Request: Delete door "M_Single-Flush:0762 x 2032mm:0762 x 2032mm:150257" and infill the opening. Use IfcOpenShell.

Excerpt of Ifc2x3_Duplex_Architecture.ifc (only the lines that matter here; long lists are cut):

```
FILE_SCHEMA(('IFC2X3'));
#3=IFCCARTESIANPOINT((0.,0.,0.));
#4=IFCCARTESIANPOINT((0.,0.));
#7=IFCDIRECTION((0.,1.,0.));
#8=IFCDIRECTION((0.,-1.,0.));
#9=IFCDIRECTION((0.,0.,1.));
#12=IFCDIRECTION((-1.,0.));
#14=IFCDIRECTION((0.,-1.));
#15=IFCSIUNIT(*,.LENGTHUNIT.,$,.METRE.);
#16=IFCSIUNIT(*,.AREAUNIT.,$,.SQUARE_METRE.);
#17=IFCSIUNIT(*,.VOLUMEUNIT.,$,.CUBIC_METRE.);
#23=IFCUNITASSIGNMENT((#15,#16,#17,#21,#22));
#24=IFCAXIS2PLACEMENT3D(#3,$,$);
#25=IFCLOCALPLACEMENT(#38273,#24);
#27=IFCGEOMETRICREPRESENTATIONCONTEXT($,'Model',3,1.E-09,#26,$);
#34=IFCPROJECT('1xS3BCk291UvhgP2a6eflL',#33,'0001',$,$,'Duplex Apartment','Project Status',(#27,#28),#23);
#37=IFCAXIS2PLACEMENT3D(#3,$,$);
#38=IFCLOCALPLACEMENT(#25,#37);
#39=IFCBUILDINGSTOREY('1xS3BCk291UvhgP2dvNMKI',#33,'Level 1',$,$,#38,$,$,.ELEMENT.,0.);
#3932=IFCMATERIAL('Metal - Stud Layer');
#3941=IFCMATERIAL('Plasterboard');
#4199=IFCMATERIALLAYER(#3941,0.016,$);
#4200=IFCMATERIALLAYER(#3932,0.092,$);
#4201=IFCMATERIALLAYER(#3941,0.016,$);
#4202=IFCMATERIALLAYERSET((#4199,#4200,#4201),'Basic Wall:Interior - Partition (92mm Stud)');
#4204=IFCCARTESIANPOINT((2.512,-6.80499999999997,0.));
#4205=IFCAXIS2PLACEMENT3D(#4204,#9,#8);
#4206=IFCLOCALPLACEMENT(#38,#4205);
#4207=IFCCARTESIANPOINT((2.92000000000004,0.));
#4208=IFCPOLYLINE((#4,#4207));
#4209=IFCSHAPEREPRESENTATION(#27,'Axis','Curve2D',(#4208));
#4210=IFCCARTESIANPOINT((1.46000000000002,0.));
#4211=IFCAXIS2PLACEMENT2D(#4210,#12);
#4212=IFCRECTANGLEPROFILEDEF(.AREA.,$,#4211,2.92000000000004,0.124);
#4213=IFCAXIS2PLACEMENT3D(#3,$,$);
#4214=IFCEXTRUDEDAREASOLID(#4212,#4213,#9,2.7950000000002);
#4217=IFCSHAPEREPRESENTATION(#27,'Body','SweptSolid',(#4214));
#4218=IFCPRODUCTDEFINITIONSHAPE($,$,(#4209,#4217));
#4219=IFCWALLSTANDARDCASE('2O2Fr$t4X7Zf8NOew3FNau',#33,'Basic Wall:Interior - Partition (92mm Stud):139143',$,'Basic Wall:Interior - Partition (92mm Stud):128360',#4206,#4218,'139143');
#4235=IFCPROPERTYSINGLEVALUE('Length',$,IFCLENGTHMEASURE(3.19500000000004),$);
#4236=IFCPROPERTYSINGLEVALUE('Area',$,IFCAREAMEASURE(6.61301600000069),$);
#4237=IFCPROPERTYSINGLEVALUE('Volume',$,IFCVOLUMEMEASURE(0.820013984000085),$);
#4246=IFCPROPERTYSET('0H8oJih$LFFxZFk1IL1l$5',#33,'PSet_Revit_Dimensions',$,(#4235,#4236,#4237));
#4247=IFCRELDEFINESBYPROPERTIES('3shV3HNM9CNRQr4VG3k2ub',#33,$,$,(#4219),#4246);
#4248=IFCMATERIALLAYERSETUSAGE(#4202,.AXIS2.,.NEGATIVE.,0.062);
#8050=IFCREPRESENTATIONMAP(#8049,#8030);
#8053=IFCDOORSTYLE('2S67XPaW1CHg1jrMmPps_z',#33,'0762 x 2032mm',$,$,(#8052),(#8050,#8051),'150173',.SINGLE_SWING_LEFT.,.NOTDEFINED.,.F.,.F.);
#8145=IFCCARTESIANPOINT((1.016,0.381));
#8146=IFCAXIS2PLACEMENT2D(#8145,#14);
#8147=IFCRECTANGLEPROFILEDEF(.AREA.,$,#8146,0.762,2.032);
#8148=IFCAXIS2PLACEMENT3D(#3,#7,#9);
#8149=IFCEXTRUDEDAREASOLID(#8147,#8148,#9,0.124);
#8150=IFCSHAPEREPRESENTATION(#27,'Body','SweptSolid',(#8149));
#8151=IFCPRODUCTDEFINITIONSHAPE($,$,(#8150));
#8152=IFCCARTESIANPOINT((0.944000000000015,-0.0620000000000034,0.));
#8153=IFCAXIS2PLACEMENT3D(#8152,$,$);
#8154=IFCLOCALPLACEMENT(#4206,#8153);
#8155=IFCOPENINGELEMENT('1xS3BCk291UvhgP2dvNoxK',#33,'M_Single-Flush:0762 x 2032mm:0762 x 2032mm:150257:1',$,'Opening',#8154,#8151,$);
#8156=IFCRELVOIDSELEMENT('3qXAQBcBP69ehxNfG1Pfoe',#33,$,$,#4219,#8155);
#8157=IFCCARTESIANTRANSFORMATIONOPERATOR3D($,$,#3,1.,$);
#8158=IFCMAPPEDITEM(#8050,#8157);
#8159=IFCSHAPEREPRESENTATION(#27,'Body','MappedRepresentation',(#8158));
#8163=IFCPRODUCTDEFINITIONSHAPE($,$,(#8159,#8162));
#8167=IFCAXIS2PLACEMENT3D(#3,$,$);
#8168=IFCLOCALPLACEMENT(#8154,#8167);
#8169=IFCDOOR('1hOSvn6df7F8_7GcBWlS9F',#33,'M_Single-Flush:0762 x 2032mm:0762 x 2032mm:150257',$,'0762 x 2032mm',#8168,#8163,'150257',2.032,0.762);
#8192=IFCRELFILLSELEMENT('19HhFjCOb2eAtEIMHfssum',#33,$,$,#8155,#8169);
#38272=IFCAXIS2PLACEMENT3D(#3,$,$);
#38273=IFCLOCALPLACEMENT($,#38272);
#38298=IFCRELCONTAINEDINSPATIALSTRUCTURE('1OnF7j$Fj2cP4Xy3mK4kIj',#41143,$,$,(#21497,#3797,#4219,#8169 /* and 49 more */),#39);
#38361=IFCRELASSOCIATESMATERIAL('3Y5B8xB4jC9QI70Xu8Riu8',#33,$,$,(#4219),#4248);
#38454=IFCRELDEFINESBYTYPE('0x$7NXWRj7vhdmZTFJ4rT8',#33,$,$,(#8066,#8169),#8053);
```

```python
import ifcopenshell
import ifcopenshell.api.feature
import ifcopenshell.api.pset
import ifcopenshell.api.root
import ifcopenshell.geom
import ifcopenshell.util.element
import ifcopenshell.util.shape
import ifcopenshell.util.unit

model = ifcopenshell.open("Ifc2x3_Duplex_Architecture.ifc")
area_scale = ifcopenshell.util.unit.calculate_unit_scale(model, "AREAUNIT")
volume_scale = ifcopenshell.util.unit.calculate_unit_scale(model, "VOLUMEUNIT")
settings = ifcopenshell.geom.settings()


def volume(element):
    """Net volume in cubic metres, openings subtracted."""
    shape = ifcopenshell.geom.create_shape(settings, element)
    return ifcopenshell.util.shape.get_volume(shape.geometry)


door = model.by_guid("1hOSvn6df7F8_7GcBWlS9F")
opening = door.FillsVoids[0].RelatingOpeningElement
wall = opening.VoidsElements[0].RelatingBuildingElement
before = volume(wall)

ifcopenshell.api.root.remove_product(model, product=door)
ifcopenshell.api.feature.remove_feature(model, feature=opening)

after = volume(wall)
thickness = 0.124  # wall thickness in metres

# Update the wall's stored quantities.
pset = model.by_id(ifcopenshell.util.element.get_pset(wall, "PSet_Revit_Dimensions", should_inherit=False)["id"])
ifcopenshell.api.pset.edit_pset(model, pset=pset, properties={
    "Area": model.create_entity("IfcAreaMeasure", after / thickness / area_scale),
    "Volume": model.create_entity("IfcVolumeMeasure", after / volume_scale),
})

print(f"wall volume {before:.3f} -> {after:.3f} m3")

model.write("Ifc2x3_Duplex_Architecture_updated.ifc")
```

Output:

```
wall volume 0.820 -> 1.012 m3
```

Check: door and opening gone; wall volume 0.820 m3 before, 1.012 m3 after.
